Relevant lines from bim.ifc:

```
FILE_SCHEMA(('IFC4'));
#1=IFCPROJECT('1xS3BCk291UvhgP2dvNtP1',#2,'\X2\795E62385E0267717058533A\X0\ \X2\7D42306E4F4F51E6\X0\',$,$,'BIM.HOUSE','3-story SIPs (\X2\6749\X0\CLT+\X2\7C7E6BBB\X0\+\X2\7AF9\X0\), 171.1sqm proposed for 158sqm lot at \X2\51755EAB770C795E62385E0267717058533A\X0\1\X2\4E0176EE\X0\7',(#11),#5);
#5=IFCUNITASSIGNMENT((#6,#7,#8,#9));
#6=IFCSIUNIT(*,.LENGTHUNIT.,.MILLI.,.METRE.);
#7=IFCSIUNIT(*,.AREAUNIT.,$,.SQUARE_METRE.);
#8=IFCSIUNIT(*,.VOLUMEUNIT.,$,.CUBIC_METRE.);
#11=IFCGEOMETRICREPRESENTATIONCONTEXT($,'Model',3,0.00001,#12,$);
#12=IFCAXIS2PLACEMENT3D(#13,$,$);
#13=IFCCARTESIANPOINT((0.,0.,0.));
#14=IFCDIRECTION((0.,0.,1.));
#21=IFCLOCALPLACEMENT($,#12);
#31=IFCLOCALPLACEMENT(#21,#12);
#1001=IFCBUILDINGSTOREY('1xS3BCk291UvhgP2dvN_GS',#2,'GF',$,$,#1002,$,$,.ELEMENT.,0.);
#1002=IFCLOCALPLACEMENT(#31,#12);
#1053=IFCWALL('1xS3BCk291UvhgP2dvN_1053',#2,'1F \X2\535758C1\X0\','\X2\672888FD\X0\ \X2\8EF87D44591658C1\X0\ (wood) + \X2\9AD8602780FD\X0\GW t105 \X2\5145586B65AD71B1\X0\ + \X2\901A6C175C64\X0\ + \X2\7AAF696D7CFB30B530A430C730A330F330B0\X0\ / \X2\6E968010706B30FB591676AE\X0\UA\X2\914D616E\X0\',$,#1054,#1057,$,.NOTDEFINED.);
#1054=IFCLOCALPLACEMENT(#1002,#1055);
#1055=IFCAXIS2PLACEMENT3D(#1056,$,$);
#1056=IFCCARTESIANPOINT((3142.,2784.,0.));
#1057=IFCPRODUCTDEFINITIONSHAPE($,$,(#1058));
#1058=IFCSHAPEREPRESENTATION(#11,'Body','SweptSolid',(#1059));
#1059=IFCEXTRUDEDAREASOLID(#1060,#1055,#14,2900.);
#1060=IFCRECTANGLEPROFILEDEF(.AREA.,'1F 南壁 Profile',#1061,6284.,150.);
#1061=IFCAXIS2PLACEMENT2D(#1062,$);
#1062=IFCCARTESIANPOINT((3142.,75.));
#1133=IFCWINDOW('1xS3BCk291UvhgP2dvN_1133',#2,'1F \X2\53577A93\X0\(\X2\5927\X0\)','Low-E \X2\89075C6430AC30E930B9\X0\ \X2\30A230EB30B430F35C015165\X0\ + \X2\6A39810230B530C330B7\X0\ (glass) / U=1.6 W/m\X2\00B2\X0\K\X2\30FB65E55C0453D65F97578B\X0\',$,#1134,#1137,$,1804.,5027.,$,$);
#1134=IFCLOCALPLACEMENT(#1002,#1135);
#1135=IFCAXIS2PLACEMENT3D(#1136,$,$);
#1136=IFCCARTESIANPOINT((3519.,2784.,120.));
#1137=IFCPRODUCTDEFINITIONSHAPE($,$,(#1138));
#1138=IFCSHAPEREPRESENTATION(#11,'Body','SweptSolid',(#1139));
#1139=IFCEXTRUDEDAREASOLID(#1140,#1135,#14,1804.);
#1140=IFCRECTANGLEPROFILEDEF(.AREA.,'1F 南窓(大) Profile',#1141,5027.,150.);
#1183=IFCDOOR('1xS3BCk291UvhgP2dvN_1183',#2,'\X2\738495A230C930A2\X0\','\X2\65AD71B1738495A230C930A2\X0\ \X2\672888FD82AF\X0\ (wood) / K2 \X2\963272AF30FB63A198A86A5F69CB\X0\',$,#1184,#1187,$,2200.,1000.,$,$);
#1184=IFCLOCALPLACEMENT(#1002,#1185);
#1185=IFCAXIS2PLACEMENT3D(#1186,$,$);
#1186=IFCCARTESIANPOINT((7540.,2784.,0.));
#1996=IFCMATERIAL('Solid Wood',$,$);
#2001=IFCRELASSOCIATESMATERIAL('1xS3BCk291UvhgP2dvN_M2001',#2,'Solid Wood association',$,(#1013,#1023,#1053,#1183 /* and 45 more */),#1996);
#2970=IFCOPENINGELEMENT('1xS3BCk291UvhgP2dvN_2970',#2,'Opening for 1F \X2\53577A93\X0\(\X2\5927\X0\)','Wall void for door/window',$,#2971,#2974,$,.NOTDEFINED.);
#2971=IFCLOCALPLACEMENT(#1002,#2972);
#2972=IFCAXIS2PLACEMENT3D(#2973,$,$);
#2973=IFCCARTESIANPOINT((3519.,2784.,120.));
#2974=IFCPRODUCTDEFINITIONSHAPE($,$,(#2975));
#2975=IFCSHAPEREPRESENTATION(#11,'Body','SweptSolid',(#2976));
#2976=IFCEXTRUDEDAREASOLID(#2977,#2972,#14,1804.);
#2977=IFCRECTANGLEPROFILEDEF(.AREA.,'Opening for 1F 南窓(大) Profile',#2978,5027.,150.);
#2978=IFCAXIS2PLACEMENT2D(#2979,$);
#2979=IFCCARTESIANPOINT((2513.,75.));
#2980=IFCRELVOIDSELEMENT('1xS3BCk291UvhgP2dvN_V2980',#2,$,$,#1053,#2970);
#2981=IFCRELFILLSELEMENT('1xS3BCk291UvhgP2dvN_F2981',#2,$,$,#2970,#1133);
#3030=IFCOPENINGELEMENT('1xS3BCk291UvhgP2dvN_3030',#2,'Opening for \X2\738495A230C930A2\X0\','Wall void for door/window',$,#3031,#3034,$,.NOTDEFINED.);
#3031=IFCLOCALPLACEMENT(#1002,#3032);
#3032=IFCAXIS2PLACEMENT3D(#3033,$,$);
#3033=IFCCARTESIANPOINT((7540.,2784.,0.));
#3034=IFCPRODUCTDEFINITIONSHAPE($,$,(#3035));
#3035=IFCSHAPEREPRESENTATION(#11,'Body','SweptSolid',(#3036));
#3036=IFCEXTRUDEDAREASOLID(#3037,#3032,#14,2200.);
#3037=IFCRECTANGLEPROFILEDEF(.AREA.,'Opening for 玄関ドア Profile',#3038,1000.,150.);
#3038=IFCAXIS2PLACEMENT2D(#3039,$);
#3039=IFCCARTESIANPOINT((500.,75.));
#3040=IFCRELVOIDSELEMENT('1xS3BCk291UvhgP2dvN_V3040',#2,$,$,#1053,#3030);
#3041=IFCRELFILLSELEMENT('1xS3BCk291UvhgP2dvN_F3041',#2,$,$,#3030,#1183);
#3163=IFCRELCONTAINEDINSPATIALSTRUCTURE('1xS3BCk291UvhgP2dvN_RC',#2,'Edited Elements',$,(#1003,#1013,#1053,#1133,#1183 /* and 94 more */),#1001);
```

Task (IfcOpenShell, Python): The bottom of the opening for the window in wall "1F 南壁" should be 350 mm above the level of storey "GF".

```python
import numpy as np
import ifcopenshell
import ifcopenshell.api.geometry
import ifcopenshell.geom
import ifcopenshell.util.element
import ifcopenshell.util.placement
import ifcopenshell.util.shape
import ifcopenshell.util.unit

model = ifcopenshell.open("bim.ifc")
unit_scale = ifcopenshell.util.unit.calculate_unit_scale(model)

window = model.by_guid("1xS3BCk291UvhgP2dvN_1133")
opening = window.FillsVoids[0].RelatingOpeningElement
storey = ifcopenshell.util.element.get_container(window, ifc_class="IfcBuildingStorey")
level = ifcopenshell.util.placement.get_local_placement(storey.ObjectPlacement)[2, 3]

# The opening's origin need not be at the sill, so measure its lowest point.
shape = ifcopenshell.geom.create_shape(ifcopenshell.geom.settings(), opening)
bottom = ifcopenshell.util.shape.get_shape_bottom_elevation(shape, shape.geometry) / unit_scale
dz = level + 0.35 / unit_scale - bottom

shift = np.array([0.0, 0.0, dz])
# The window is not placed relative to its opening, so move both.
for product in (opening, window):
    matrix = ifcopenshell.util.placement.get_local_placement(product.ObjectPlacement)
    matrix[:3, 3] += shift
    ifcopenshell.api.geometry.edit_object_placement(model, product=product, matrix=matrix, is_si=False)

print(f"moved by {dz * unit_scale:+.3f} m")

model.write("bim_updated.ifc")
```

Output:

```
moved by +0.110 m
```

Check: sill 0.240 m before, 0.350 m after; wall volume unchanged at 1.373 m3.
